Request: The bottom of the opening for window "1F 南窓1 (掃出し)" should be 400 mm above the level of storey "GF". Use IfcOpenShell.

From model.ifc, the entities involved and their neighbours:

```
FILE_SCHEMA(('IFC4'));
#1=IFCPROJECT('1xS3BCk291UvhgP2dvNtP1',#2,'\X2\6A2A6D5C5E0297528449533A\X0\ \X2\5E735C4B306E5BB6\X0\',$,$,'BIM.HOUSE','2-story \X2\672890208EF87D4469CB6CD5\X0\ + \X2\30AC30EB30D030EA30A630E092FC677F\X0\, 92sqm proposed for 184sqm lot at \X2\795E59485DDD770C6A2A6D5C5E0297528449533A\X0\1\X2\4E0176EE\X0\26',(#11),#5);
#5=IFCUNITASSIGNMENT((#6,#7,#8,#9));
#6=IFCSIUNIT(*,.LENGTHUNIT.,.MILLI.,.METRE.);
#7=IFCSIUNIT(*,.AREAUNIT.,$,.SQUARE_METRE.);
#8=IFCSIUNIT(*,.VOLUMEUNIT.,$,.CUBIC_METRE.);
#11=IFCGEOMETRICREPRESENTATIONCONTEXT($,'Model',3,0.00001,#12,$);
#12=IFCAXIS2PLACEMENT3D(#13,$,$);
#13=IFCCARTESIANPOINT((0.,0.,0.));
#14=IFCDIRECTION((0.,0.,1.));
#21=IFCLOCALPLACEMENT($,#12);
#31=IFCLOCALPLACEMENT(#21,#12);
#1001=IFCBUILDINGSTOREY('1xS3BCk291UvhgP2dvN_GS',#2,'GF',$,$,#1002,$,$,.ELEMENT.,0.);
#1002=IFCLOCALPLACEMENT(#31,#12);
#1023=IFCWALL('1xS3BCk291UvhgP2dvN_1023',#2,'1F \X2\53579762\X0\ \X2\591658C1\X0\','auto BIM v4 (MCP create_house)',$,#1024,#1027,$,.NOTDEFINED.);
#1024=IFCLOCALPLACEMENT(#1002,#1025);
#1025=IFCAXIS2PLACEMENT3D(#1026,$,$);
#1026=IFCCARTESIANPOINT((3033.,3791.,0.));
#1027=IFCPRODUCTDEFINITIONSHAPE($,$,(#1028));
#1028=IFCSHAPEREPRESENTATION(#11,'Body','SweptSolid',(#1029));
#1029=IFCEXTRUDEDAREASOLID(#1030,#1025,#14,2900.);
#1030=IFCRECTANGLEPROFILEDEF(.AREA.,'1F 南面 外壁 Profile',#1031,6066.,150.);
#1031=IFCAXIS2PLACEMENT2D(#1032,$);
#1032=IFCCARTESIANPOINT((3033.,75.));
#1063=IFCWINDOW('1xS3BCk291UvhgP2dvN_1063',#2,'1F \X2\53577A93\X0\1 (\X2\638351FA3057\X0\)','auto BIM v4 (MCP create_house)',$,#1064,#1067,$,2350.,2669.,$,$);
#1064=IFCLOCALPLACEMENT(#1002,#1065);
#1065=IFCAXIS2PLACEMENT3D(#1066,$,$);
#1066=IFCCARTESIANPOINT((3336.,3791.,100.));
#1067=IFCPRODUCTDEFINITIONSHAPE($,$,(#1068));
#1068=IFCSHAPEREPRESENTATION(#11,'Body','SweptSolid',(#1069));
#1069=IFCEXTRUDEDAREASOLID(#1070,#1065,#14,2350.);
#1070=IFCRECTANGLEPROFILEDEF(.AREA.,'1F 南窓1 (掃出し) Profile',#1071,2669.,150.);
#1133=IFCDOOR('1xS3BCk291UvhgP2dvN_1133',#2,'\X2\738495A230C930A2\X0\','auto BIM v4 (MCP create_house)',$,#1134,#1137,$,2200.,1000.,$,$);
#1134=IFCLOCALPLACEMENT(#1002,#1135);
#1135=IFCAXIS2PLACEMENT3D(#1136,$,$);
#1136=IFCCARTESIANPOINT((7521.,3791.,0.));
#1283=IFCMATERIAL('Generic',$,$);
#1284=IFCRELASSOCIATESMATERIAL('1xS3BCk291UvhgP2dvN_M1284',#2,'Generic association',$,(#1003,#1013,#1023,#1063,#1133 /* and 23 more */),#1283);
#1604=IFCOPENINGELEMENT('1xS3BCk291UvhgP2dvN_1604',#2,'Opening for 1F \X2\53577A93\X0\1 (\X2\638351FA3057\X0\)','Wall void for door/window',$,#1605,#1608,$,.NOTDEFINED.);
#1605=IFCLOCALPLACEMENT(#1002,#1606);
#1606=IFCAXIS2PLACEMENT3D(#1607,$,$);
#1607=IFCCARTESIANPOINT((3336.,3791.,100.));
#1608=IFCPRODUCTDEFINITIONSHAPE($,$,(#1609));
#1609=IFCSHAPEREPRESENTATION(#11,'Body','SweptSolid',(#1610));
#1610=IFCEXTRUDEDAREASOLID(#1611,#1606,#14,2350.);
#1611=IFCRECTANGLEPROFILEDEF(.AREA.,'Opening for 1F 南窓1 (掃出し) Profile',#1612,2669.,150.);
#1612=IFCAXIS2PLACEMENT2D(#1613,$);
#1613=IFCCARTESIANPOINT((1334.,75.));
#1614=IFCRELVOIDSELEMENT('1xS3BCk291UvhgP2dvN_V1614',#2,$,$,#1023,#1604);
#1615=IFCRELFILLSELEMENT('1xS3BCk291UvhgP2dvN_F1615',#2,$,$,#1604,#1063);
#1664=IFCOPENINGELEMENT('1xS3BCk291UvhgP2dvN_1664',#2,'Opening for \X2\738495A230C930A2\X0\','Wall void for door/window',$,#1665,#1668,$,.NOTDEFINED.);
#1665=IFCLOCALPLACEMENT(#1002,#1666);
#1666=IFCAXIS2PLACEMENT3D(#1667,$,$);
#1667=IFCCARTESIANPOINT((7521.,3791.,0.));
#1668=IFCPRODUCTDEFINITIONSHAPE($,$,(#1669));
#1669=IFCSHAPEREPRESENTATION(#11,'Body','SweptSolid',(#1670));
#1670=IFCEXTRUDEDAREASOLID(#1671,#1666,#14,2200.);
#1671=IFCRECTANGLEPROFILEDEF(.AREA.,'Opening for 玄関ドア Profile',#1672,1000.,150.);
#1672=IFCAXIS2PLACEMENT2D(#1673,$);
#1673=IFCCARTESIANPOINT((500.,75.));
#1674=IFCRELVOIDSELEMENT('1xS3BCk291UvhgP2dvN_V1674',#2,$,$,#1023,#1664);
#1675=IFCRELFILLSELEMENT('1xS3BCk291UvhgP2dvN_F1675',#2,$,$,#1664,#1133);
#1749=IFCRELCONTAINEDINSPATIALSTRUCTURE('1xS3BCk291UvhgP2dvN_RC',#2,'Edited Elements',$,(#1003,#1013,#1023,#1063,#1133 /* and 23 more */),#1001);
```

```python
import numpy as np
import ifcopenshell
import ifcopenshell.api.geometry
import ifcopenshell.geom
import ifcopenshell.util.element
import ifcopenshell.util.placement
import ifcopenshell.util.shape
import ifcopenshell.util.unit

model = ifcopenshell.open("model.ifc")
unit_scale = ifcopenshell.util.unit.calculate_unit_scale(model)

window = model.by_guid("1xS3BCk291UvhgP2dvN_1063")
opening = window.FillsVoids[0].RelatingOpeningElement
storey = ifcopenshell.util.element.get_container(window, ifc_class="IfcBuildingStorey")
level = ifcopenshell.util.placement.get_local_placement(storey.ObjectPlacement)[2, 3]

# The opening's origin need not be at the sill, so measure its lowest point.
shape = ifcopenshell.geom.create_shape(ifcopenshell.geom.settings(), opening)
bottom = ifcopenshell.util.shape.get_shape_bottom_elevation(shape, shape.geometry) / unit_scale
dz = level + 400.0 - bottom

shift = np.array([0.0, 0.0, dz])
# The window is not placed relative to its opening, so move both.
for product in (opening, window):
    matrix = ifcopenshell.util.placement.get_local_placement(product.ObjectPlacement)
    matrix[:3, 3] += shift
    ifcopenshell.api.geometry.edit_object_placement(model, product=product, matrix=matrix, is_si=False)

print(f"moved by {dz * unit_scale:+.3f} m")

model.write("model_v2.ifc")
```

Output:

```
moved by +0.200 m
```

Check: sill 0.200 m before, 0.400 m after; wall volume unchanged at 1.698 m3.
